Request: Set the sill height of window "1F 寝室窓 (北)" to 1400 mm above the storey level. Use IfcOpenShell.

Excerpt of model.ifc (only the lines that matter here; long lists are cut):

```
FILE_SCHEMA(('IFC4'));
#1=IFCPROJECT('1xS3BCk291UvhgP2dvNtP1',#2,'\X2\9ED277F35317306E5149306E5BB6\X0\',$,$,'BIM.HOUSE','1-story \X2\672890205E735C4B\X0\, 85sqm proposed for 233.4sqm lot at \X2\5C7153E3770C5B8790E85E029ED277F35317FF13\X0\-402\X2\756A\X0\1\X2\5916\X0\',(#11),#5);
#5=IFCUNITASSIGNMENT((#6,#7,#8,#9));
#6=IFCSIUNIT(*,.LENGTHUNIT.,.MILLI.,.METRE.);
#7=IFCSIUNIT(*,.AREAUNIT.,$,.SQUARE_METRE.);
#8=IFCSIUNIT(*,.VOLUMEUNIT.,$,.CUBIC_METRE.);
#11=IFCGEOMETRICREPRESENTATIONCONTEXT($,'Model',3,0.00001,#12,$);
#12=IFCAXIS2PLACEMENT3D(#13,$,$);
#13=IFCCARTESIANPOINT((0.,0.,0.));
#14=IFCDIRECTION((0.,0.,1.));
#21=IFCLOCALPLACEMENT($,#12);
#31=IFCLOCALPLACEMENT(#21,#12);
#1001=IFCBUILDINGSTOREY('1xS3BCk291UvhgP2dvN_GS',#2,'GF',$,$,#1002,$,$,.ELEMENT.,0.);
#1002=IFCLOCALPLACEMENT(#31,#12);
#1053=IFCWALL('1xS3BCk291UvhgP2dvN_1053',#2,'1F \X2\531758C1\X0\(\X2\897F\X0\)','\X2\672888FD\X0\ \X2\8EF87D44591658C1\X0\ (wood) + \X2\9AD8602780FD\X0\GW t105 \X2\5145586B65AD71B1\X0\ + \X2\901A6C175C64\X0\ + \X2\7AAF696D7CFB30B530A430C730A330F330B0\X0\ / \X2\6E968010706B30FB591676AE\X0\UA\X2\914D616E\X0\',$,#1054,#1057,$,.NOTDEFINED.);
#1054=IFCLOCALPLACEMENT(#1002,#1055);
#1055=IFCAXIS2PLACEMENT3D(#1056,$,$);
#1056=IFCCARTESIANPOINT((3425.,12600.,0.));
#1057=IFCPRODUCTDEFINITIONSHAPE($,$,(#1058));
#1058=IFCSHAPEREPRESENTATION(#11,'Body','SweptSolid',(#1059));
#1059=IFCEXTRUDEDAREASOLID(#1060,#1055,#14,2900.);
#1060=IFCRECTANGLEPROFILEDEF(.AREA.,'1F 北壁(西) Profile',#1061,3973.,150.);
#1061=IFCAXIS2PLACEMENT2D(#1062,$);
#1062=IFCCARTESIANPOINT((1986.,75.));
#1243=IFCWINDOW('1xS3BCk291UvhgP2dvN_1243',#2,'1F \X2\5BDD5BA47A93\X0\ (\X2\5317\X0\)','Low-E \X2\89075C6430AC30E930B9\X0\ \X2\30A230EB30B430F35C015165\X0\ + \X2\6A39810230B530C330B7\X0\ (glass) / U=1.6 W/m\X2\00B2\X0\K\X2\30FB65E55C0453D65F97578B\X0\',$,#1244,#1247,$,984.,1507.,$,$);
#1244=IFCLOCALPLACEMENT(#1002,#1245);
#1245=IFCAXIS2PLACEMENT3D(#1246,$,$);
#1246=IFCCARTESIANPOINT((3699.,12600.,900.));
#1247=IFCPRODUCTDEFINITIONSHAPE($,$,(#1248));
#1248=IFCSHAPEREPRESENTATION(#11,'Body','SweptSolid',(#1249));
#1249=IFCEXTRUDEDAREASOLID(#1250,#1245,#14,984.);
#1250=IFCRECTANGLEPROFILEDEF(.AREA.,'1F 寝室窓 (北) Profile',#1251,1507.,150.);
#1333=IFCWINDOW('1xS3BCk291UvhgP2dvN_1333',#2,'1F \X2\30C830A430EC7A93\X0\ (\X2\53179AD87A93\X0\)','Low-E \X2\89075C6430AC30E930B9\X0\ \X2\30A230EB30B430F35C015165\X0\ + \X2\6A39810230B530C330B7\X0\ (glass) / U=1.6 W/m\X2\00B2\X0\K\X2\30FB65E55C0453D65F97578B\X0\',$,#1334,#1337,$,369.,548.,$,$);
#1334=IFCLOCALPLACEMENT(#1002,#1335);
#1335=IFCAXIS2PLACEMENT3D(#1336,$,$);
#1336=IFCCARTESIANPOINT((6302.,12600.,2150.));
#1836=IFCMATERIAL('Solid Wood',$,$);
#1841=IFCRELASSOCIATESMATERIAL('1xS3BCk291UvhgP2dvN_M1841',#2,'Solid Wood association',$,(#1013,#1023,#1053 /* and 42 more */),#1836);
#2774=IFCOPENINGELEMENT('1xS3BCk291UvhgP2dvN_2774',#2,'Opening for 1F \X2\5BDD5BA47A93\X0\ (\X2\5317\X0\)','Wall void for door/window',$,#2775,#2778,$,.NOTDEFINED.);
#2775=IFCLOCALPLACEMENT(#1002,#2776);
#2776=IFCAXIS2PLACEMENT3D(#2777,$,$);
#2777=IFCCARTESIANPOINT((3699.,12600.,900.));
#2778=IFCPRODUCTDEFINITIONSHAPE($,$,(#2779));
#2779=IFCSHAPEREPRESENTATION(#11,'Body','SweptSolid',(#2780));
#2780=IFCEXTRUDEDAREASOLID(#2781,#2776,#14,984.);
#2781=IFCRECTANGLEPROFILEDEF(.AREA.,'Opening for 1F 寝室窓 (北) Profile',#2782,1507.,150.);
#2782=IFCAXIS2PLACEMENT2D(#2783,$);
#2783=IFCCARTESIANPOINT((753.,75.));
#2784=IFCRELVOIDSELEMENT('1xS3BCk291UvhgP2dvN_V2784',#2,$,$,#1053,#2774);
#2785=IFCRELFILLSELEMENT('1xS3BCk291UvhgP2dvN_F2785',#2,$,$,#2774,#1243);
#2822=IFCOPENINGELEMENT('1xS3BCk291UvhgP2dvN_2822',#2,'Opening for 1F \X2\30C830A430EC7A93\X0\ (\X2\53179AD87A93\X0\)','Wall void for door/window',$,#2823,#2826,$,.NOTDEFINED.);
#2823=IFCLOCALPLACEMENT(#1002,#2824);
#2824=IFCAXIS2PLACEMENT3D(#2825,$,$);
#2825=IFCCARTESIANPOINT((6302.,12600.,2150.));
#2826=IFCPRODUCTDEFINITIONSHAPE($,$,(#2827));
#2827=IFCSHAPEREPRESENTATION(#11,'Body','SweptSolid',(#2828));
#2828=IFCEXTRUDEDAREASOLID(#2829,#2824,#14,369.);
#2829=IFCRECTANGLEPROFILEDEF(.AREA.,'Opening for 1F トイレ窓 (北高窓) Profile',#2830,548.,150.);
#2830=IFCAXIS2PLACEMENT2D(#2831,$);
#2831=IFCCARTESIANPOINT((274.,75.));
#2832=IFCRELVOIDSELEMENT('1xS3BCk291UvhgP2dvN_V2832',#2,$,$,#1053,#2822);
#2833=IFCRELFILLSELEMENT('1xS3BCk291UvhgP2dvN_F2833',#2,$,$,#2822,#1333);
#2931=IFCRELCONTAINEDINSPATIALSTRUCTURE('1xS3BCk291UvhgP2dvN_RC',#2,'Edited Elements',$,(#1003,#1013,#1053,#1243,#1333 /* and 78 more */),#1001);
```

```python
import numpy as np
import ifcopenshell
import ifcopenshell.api.geometry
import ifcopenshell.geom
import ifcopenshell.util.element
import ifcopenshell.util.placement
import ifcopenshell.util.shape
import ifcopenshell.util.unit

model = ifcopenshell.open("model.ifc")
unit_scale = ifcopenshell.util.unit.calculate_unit_scale(model)

window = model.by_guid("1xS3BCk291UvhgP2dvN_1243")
opening = window.FillsVoids[0].RelatingOpeningElement
storey = ifcopenshell.util.element.get_container(window, ifc_class="IfcBuildingStorey")
level = ifcopenshell.util.placement.get_local_placement(storey.ObjectPlacement)[2, 3]

# The opening's origin need not be at the sill, so measure its lowest point.
shape = ifcopenshell.geom.create_shape(ifcopenshell.geom.settings(), opening)
bottom = ifcopenshell.util.shape.get_shape_bottom_elevation(shape, shape.geometry) / unit_scale
dz = level + 1.4 / unit_scale - bottom

shift = np.array([0.0, 0.0, dz])
# The window is not placed relative to its opening, so move both.
for product in (opening, window):
    matrix = ifcopenshell.util.placement.get_local_placement(product.ObjectPlacement)
    matrix[:3, 3] += shift
    ifcopenshell.api.geometry.edit_object_placement(model, product=product, matrix=matrix, is_si=False)

print(f"moved by {dz * unit_scale:+.3f} m")

model.write("model_v2.ifc")
```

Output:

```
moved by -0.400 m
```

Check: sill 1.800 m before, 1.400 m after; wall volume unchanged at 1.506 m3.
